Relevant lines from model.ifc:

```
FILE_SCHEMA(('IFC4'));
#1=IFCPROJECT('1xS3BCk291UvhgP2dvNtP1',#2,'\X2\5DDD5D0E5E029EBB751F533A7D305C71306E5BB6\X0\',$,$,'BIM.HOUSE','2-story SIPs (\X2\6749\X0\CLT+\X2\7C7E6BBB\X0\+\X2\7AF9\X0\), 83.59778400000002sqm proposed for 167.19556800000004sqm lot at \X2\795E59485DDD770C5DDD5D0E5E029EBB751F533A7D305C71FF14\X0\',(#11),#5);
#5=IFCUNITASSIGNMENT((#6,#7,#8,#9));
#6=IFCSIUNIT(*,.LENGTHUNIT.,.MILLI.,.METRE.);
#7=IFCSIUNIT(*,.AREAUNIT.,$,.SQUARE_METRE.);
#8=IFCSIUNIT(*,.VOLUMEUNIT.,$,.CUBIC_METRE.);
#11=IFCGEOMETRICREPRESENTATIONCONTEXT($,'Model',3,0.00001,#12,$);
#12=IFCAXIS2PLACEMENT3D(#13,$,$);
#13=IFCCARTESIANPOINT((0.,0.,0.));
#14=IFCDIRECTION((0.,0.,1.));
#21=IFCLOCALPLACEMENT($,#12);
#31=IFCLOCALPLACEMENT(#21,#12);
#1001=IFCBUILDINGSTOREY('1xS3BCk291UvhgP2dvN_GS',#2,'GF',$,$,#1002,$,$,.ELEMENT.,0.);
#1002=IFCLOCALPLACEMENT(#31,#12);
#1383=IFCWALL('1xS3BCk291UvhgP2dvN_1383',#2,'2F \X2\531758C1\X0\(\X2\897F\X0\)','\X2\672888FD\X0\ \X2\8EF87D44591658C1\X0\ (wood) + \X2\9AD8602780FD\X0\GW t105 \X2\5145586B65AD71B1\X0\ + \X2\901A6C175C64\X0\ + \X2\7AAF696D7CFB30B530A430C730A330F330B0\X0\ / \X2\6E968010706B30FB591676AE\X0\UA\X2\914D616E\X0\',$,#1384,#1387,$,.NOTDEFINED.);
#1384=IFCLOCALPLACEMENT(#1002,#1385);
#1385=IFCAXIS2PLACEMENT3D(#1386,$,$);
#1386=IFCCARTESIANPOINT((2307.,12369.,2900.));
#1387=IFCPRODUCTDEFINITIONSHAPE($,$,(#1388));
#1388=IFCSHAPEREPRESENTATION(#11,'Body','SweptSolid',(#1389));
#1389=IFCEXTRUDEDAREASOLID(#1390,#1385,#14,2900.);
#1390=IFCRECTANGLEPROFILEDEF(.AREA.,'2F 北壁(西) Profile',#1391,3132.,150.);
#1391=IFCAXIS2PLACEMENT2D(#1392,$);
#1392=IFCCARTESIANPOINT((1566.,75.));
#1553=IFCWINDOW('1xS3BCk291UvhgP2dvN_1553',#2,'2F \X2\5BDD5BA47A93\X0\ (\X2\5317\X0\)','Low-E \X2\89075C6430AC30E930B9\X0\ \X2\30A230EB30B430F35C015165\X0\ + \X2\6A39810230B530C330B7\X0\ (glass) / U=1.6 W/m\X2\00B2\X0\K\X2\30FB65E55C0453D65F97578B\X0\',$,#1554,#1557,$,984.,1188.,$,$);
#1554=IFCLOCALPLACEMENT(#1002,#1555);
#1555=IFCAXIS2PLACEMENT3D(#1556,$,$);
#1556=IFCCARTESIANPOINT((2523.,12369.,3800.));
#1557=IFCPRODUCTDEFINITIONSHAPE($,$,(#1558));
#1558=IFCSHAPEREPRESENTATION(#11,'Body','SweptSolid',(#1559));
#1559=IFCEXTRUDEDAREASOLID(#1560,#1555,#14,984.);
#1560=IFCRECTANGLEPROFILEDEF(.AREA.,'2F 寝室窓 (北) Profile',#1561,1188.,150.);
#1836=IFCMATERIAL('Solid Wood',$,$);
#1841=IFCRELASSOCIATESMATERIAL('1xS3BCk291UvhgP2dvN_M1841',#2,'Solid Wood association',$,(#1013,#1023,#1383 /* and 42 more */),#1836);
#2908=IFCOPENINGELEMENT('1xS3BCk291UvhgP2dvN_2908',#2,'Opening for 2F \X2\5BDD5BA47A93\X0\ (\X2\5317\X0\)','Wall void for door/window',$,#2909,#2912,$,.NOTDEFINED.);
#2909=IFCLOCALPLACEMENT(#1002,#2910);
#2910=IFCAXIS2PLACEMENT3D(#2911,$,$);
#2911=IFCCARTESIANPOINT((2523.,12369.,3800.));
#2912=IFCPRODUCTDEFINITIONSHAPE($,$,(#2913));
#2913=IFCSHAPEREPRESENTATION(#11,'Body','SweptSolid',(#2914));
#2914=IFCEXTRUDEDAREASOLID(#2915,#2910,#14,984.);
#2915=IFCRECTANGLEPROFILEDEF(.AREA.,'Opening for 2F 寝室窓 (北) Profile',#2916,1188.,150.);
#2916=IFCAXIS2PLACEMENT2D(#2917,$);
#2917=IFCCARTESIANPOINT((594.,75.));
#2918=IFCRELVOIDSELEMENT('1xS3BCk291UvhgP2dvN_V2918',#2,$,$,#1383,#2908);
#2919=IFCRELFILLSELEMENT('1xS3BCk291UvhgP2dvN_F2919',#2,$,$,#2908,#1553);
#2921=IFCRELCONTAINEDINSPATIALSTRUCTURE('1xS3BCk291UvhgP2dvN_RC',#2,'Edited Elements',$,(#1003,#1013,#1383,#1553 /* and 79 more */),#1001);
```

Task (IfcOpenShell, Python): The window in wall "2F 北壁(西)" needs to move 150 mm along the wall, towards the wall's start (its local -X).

```python
import ifcopenshell
import ifcopenshell.api.geometry
import ifcopenshell.util.placement
import ifcopenshell.util.unit

model = ifcopenshell.open("model.ifc")
unit_scale = ifcopenshell.util.unit.calculate_unit_scale(model)

window = model.by_guid("1xS3BCk291UvhgP2dvN_1553")
opening = window.FillsVoids[0].RelatingOpeningElement
wall = opening.VoidsElements[0].RelatingBuildingElement

wall_matrix = ifcopenshell.util.placement.get_local_placement(wall.ObjectPlacement)
shift = wall_matrix[:3, 0] * -0.15 / unit_scale
before = ifcopenshell.util.placement.get_local_placement(window.ObjectPlacement)[:3, 3].copy()

# The window is not placed relative to its opening, so move both.
for product in (opening, window):
    matrix = ifcopenshell.util.placement.get_local_placement(product.ObjectPlacement)
    matrix[:3, 3] += shift
    ifcopenshell.api.geometry.edit_object_placement(model, product=product, matrix=matrix, is_si=False)

after = ifcopenshell.util.placement.get_local_placement(window.ObjectPlacement)[:3, 3]
print("window moved by", (after - before).round(3) + 0.0)

model.write("model-out.ifc")
```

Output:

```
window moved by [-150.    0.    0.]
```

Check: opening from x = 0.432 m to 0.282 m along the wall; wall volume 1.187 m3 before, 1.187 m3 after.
